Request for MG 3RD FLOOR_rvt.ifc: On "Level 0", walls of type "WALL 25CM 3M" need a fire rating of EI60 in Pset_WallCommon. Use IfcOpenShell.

First a look at what the model holds.

```python
import ifcopenshell
import ifcopenshell.util.element

model = ifcopenshell.open("MG 3RD FLOOR_rvt.ifc")
print(model.schema)
storey = next(s for s in model.by_type("IfcBuildingStorey") if s.Name == "Level 0")
walls = [e for e in ifcopenshell.util.element.get_decomposition(storey) if e.is_a("IfcWall")]
seen = {}
for e in walls:
    element_type = ifcopenshell.util.element.get_type(e)
    key = (element_type.Name if element_type != e and element_type else None, ifcopenshell.util.element.get_pset(e, "Pset_WallCommon", "FireRating"))
    seen[key] = seen.get(key, 0) + 1
for (name, value), count in sorted(seen.items(), key=str):
    print(count, "x", name, "|", value)
```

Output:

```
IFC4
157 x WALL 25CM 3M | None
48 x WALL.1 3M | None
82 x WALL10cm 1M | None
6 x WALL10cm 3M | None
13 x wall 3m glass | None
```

```python
import ifcopenshell
import ifcopenshell.api.pset
import ifcopenshell.util.element

model = ifcopenshell.open("MG 3RD FLOOR_rvt.ifc")

storey = next(s for s in model.by_type("IfcBuildingStorey") if s.Name == "Level 0")
walls = [e for e in ifcopenshell.util.element.get_decomposition(storey) if e.is_a("IfcWall")]

count = 0
for e in walls:
    element_type = ifcopenshell.util.element.get_type(e)
    if element_type in (None, e) or element_type.Name != "WALL 25CM 3M":
        continue
    # add_pset returns the element's existing set when there is one.
    pset = ifcopenshell.api.pset.add_pset(model, product=e, name="Pset_WallCommon")
    ifcopenshell.api.pset.edit_pset(model, pset=pset, properties={"FireRating": "EI60"})
    count += 1

print(count, "walls updated")

model.write("MG 3RD FLOOR_rvt_rev.ifc")
```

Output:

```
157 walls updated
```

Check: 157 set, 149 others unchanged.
